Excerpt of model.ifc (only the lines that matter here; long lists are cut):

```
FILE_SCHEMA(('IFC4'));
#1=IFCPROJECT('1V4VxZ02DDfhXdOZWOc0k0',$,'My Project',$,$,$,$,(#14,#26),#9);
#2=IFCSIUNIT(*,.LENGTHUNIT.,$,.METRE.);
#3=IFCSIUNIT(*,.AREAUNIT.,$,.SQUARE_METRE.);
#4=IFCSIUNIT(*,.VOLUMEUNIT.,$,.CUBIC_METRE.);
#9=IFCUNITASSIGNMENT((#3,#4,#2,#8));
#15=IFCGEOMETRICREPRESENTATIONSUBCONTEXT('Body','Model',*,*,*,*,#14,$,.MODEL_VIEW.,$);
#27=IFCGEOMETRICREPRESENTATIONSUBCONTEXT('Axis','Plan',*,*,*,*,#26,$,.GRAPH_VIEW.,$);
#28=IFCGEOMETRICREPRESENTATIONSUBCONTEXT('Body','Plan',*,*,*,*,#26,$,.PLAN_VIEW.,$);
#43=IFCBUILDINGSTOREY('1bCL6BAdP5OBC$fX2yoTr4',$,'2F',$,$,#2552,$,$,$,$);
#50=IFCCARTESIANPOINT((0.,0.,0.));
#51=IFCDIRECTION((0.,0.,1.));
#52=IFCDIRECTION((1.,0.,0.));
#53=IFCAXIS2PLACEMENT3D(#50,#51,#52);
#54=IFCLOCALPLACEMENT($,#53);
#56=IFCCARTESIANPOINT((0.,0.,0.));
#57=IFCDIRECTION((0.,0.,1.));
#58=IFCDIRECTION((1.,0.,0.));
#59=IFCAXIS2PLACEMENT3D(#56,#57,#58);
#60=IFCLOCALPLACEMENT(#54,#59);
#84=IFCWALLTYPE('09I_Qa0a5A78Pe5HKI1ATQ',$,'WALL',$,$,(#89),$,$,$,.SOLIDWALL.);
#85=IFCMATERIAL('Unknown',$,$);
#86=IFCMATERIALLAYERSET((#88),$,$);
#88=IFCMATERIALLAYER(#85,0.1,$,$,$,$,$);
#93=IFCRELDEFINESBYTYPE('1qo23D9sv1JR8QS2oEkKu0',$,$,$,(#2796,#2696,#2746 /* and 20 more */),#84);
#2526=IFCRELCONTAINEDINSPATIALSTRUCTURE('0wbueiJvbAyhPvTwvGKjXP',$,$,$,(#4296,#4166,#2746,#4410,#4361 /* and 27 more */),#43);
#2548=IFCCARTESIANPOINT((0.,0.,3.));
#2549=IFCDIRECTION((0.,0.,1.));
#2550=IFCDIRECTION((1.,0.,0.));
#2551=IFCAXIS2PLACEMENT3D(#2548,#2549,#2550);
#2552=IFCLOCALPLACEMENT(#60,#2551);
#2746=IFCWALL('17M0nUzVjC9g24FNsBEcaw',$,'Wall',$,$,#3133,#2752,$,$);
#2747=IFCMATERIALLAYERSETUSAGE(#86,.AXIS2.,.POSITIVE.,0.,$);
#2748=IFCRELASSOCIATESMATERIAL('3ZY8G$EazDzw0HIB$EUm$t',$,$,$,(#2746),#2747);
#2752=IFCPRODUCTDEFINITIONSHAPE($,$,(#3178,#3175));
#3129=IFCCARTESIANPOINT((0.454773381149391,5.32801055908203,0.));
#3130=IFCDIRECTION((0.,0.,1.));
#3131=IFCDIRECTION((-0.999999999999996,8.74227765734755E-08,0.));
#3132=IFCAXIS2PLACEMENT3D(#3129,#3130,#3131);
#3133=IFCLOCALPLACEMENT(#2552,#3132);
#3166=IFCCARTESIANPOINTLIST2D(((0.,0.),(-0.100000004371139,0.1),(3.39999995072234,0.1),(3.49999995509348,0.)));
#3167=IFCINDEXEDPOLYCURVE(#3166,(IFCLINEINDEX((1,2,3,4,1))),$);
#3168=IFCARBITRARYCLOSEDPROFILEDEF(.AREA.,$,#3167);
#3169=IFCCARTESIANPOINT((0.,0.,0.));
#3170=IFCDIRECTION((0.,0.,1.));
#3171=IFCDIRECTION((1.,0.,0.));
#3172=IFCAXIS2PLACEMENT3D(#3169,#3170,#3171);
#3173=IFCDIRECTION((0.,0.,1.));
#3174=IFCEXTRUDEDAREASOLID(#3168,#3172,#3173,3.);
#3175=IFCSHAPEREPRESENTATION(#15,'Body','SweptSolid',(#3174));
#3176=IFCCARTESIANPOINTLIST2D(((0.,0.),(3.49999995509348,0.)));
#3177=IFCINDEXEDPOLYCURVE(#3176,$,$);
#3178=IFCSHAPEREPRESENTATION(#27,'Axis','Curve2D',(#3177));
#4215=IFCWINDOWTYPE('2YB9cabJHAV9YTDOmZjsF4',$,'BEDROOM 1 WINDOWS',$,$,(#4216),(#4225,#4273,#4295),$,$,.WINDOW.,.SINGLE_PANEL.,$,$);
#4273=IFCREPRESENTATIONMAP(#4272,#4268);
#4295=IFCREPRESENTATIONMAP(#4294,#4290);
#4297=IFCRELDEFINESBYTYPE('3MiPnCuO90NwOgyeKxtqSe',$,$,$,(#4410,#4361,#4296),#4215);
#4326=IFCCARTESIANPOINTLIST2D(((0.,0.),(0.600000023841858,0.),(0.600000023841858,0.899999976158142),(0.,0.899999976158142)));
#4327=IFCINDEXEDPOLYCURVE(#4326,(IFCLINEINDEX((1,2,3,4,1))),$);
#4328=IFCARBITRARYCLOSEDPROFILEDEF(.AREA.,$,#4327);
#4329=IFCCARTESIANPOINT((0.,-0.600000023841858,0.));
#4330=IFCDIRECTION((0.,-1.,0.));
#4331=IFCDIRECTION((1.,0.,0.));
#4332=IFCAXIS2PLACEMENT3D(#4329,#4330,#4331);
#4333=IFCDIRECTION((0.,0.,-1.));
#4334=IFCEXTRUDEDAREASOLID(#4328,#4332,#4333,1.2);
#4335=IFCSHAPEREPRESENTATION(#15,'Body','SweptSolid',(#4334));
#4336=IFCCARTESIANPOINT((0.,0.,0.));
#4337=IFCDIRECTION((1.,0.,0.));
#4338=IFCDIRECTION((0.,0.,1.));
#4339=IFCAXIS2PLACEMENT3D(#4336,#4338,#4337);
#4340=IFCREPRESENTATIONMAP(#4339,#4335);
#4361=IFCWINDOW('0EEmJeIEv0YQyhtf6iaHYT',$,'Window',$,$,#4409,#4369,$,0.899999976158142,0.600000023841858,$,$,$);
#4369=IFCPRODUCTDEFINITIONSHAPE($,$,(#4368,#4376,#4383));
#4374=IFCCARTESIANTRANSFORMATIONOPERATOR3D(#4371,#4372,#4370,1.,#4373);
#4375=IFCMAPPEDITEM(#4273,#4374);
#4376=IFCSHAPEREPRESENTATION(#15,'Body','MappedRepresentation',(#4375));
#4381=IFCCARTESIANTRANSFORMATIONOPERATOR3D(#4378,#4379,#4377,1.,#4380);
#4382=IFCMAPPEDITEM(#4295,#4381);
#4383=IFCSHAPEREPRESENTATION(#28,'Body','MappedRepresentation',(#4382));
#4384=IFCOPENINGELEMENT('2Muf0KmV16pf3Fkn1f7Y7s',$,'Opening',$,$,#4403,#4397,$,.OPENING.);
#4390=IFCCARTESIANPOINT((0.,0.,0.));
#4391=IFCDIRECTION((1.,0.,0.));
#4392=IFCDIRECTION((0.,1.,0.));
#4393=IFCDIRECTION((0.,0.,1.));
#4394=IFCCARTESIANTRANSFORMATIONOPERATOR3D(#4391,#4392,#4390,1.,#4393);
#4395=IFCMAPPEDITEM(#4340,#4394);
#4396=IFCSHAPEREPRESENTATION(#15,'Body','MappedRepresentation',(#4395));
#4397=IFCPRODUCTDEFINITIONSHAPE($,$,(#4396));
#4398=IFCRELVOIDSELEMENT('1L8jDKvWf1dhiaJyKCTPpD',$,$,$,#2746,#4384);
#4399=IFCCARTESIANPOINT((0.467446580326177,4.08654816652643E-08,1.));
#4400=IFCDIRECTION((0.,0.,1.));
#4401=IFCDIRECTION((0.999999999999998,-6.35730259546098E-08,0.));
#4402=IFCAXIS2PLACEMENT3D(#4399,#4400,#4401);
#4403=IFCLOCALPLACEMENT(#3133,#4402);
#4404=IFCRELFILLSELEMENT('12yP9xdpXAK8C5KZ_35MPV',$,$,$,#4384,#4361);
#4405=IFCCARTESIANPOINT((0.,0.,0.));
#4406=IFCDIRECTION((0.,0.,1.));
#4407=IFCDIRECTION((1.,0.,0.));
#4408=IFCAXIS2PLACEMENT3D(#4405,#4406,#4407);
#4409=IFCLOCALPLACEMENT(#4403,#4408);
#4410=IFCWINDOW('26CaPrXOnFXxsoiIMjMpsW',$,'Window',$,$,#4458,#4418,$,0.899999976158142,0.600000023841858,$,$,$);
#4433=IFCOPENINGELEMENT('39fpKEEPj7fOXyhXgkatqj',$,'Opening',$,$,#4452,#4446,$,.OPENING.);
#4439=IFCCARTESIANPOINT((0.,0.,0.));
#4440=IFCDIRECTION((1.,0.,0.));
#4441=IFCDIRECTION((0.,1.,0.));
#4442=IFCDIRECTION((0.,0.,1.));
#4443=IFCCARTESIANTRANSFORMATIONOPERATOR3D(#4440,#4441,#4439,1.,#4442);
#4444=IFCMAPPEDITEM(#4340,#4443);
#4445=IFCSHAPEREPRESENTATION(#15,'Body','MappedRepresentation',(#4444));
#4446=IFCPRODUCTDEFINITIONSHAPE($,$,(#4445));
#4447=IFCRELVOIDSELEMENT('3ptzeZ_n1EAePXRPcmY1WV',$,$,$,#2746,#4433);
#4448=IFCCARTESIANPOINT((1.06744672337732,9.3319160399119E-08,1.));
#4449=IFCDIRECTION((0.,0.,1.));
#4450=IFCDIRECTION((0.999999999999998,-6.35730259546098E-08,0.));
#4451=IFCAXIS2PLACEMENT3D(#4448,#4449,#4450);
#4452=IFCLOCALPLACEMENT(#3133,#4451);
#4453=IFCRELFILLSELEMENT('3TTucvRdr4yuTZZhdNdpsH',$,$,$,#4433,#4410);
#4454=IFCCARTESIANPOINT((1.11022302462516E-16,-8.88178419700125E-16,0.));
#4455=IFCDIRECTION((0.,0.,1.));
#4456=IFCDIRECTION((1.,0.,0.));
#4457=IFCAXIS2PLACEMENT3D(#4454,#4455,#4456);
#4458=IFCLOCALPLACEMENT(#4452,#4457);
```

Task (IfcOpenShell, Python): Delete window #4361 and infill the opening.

```python
import ifcopenshell
import ifcopenshell.api.feature
import ifcopenshell.api.root
import ifcopenshell.geom
import ifcopenshell.util.shape

model = ifcopenshell.open("model.ifc")
settings = ifcopenshell.geom.settings()


def volume(element):
    """Net volume in cubic metres, openings subtracted."""
    shape = ifcopenshell.geom.create_shape(settings, element)
    return ifcopenshell.util.shape.get_volume(shape.geometry)


window = model.by_guid("0EEmJeIEv0YQyhtf6iaHYT")
opening = window.FillsVoids[0].RelatingOpeningElement
wall = opening.VoidsElements[0].RelatingBuildingElement
before = volume(wall)

ifcopenshell.api.root.remove_product(model, product=window)
ifcopenshell.api.feature.remove_feature(model, feature=opening)

after = volume(wall)

print(f"wall volume {before:.3f} -> {after:.3f} m3")

model.write("model-out.ifc")
```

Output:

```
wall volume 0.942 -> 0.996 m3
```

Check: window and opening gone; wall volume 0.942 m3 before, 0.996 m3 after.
